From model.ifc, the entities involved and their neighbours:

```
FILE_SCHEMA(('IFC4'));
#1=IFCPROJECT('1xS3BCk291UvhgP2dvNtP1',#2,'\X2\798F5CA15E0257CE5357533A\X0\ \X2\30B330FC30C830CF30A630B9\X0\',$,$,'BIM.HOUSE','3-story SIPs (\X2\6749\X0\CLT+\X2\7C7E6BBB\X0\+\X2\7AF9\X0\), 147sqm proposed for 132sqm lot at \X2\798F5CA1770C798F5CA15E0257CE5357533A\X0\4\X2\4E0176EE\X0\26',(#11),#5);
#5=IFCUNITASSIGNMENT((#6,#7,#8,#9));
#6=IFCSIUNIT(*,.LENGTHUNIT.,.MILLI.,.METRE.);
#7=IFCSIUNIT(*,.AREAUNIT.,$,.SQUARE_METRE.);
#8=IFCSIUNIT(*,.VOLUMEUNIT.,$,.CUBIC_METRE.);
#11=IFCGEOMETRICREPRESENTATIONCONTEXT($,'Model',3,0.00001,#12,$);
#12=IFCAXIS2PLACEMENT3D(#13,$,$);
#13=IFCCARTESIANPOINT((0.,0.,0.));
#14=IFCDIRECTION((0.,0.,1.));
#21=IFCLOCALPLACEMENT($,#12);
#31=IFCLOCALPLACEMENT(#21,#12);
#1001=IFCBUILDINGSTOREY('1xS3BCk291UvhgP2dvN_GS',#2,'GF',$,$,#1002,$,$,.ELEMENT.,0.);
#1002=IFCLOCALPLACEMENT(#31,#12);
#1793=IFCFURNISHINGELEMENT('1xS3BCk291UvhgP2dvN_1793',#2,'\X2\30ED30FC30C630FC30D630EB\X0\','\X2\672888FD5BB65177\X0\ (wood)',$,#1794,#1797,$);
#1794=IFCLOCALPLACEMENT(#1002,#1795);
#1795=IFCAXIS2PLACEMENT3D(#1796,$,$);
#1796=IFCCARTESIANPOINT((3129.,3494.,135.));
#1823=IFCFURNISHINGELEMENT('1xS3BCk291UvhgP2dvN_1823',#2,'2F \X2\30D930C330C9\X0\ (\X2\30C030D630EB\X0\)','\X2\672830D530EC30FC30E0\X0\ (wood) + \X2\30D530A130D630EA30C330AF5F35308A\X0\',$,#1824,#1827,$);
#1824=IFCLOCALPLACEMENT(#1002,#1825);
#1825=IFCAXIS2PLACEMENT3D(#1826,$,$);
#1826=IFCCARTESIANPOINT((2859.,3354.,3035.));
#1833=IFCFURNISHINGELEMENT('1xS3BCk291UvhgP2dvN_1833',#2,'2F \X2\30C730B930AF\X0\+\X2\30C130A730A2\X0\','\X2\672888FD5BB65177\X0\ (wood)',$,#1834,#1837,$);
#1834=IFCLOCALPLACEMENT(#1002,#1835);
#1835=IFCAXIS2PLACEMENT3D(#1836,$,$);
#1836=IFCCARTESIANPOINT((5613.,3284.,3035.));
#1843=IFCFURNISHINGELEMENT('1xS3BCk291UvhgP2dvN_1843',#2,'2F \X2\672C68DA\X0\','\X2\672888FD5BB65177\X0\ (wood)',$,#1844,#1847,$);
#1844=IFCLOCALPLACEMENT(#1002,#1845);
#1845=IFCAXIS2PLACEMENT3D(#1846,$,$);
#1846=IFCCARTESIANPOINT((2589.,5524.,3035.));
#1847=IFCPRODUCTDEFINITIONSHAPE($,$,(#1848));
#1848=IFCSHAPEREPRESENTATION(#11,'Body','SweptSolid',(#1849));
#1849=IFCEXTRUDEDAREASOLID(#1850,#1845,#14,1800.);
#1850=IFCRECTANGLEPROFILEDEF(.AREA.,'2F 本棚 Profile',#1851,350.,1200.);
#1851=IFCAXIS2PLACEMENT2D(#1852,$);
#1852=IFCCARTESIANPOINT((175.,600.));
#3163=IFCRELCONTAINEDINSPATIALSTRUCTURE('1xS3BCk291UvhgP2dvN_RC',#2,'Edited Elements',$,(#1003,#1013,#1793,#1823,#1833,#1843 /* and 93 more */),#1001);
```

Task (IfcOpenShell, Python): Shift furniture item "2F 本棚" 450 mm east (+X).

```python
import ifcopenshell
import ifcopenshell.api.geometry
import ifcopenshell.util.placement

model = ifcopenshell.open("model.ifc")

item = model.by_id(1843)
matrix = ifcopenshell.util.placement.get_local_placement(item.ObjectPlacement)
matrix[0, 3] += 450.0
ifcopenshell.api.geometry.edit_object_placement(model, product=item, matrix=matrix, is_si=False)

print(ifcopenshell.util.placement.get_local_placement(item.ObjectPlacement).round(3) + 0.0)

model.write("model_v2.ifc")
```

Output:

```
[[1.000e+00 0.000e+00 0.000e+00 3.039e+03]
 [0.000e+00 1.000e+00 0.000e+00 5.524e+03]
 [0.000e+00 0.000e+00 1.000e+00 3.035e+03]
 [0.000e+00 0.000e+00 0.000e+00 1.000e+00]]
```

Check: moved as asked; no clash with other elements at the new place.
